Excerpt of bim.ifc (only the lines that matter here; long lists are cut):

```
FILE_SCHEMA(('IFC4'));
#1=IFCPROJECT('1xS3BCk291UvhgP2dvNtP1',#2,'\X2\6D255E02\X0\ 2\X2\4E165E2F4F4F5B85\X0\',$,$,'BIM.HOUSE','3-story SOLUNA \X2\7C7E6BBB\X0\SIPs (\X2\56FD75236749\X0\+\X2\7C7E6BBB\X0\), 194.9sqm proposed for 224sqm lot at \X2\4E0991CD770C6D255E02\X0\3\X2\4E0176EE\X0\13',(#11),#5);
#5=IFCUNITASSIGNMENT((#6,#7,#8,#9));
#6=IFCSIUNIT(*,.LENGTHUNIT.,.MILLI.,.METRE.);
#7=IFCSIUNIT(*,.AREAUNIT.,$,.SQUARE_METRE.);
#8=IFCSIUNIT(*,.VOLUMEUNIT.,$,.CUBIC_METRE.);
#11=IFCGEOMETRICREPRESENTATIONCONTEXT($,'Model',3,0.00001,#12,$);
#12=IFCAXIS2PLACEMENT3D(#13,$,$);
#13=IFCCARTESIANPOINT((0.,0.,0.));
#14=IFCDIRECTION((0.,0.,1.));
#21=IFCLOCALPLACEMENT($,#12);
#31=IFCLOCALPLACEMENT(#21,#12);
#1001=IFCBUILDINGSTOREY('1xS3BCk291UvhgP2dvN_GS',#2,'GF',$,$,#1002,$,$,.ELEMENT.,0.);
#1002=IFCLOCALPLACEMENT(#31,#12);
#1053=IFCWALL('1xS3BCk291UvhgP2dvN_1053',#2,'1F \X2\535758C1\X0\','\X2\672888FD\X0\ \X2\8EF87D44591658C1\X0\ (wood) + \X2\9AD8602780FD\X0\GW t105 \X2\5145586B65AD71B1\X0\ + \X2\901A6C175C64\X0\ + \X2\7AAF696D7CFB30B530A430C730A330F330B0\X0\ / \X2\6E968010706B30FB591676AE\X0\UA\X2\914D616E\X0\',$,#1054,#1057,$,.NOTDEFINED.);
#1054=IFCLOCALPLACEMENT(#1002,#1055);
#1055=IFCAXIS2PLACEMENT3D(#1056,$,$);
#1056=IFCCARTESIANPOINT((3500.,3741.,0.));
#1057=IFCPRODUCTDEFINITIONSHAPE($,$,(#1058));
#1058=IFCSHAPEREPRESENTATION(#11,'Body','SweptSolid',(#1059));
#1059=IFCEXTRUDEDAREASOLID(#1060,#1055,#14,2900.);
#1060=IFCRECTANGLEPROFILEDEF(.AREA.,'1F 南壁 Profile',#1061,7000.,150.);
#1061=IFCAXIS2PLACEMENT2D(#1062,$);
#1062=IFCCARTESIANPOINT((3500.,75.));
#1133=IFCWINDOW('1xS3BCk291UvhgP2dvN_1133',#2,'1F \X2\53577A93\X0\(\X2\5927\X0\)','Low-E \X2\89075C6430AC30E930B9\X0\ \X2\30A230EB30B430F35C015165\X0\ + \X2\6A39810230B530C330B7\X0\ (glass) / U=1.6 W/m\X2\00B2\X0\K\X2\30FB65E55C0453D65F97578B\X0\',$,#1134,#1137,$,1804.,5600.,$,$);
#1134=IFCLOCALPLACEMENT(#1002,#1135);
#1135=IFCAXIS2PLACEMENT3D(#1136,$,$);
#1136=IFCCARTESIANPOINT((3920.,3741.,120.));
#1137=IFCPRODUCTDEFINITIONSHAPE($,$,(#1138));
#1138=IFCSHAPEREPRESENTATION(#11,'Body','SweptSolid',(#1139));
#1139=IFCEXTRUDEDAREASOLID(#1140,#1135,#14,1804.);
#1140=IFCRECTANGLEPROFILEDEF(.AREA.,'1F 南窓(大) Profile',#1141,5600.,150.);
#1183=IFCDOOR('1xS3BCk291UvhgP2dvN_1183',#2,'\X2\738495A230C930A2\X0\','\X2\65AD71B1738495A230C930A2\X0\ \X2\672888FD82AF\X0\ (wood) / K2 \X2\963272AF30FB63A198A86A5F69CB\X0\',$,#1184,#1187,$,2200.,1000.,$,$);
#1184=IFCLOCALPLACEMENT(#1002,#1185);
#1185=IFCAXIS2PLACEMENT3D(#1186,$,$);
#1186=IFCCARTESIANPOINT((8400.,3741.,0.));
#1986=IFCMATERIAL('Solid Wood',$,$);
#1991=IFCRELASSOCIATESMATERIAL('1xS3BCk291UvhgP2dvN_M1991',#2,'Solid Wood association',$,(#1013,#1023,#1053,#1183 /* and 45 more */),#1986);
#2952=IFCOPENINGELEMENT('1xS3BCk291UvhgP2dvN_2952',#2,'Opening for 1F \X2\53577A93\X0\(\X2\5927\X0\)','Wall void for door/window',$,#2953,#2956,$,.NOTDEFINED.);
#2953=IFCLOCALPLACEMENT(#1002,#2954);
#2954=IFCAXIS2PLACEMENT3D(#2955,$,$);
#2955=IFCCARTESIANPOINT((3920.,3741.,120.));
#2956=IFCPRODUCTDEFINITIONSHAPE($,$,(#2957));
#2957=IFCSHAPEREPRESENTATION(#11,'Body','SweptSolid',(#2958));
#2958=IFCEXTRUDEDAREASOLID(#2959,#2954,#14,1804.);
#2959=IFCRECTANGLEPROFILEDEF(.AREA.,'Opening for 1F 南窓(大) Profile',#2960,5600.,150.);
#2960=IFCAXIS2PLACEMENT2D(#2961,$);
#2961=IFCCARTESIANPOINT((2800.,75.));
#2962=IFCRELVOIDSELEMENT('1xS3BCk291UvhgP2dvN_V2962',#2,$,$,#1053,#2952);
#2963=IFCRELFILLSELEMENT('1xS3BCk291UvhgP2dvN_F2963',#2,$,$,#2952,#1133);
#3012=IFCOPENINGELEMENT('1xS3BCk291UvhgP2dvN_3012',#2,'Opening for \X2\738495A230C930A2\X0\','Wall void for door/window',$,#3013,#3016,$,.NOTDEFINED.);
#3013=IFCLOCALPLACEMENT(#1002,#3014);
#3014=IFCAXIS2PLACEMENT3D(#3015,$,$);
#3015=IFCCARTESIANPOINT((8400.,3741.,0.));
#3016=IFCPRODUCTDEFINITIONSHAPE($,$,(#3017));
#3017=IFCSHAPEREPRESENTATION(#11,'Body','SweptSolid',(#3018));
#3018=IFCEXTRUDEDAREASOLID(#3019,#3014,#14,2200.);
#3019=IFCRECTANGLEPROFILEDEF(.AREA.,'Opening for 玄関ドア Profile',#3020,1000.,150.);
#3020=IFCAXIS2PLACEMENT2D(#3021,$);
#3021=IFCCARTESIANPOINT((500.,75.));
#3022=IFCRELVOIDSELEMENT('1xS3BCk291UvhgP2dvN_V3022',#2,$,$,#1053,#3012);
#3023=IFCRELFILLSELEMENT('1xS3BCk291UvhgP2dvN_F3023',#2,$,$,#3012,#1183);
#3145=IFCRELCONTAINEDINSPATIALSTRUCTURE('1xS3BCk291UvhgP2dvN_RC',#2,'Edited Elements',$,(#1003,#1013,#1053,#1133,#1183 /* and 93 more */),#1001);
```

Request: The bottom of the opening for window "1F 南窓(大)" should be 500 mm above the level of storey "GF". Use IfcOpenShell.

```python
import numpy as np
import ifcopenshell
import ifcopenshell.api.geometry
import ifcopenshell.geom
import ifcopenshell.util.element
import ifcopenshell.util.placement
import ifcopenshell.util.shape
import ifcopenshell.util.unit

model = ifcopenshell.open("bim.ifc")
unit_scale = ifcopenshell.util.unit.calculate_unit_scale(model)

window = model.by_id(1133)
opening = window.FillsVoids[0].RelatingOpeningElement
storey = ifcopenshell.util.element.get_container(window, ifc_class="IfcBuildingStorey")
level = ifcopenshell.util.placement.get_local_placement(storey.ObjectPlacement)[2, 3]

# The opening's origin need not be at the sill, so measure its lowest point.
shape = ifcopenshell.geom.create_shape(ifcopenshell.geom.settings(), opening)
bottom = ifcopenshell.util.shape.get_shape_bottom_elevation(shape, shape.geometry) / unit_scale
dz = level + 0.5 / unit_scale - bottom

shift = np.array([0.0, 0.0, dz])
# The window is not placed relative to its opening, so move both.
for product in (opening, window):
    matrix = ifcopenshell.util.placement.get_local_placement(product.ObjectPlacement)
    matrix[:3, 3] += shift
    ifcopenshell.api.geometry.edit_object_placement(model, product=product, matrix=matrix, is_si=False)

print(f"moved by {dz * unit_scale:+.3f} m")

model.write("bim_rev.ifc")
```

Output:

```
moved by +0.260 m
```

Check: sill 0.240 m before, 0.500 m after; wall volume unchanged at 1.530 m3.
